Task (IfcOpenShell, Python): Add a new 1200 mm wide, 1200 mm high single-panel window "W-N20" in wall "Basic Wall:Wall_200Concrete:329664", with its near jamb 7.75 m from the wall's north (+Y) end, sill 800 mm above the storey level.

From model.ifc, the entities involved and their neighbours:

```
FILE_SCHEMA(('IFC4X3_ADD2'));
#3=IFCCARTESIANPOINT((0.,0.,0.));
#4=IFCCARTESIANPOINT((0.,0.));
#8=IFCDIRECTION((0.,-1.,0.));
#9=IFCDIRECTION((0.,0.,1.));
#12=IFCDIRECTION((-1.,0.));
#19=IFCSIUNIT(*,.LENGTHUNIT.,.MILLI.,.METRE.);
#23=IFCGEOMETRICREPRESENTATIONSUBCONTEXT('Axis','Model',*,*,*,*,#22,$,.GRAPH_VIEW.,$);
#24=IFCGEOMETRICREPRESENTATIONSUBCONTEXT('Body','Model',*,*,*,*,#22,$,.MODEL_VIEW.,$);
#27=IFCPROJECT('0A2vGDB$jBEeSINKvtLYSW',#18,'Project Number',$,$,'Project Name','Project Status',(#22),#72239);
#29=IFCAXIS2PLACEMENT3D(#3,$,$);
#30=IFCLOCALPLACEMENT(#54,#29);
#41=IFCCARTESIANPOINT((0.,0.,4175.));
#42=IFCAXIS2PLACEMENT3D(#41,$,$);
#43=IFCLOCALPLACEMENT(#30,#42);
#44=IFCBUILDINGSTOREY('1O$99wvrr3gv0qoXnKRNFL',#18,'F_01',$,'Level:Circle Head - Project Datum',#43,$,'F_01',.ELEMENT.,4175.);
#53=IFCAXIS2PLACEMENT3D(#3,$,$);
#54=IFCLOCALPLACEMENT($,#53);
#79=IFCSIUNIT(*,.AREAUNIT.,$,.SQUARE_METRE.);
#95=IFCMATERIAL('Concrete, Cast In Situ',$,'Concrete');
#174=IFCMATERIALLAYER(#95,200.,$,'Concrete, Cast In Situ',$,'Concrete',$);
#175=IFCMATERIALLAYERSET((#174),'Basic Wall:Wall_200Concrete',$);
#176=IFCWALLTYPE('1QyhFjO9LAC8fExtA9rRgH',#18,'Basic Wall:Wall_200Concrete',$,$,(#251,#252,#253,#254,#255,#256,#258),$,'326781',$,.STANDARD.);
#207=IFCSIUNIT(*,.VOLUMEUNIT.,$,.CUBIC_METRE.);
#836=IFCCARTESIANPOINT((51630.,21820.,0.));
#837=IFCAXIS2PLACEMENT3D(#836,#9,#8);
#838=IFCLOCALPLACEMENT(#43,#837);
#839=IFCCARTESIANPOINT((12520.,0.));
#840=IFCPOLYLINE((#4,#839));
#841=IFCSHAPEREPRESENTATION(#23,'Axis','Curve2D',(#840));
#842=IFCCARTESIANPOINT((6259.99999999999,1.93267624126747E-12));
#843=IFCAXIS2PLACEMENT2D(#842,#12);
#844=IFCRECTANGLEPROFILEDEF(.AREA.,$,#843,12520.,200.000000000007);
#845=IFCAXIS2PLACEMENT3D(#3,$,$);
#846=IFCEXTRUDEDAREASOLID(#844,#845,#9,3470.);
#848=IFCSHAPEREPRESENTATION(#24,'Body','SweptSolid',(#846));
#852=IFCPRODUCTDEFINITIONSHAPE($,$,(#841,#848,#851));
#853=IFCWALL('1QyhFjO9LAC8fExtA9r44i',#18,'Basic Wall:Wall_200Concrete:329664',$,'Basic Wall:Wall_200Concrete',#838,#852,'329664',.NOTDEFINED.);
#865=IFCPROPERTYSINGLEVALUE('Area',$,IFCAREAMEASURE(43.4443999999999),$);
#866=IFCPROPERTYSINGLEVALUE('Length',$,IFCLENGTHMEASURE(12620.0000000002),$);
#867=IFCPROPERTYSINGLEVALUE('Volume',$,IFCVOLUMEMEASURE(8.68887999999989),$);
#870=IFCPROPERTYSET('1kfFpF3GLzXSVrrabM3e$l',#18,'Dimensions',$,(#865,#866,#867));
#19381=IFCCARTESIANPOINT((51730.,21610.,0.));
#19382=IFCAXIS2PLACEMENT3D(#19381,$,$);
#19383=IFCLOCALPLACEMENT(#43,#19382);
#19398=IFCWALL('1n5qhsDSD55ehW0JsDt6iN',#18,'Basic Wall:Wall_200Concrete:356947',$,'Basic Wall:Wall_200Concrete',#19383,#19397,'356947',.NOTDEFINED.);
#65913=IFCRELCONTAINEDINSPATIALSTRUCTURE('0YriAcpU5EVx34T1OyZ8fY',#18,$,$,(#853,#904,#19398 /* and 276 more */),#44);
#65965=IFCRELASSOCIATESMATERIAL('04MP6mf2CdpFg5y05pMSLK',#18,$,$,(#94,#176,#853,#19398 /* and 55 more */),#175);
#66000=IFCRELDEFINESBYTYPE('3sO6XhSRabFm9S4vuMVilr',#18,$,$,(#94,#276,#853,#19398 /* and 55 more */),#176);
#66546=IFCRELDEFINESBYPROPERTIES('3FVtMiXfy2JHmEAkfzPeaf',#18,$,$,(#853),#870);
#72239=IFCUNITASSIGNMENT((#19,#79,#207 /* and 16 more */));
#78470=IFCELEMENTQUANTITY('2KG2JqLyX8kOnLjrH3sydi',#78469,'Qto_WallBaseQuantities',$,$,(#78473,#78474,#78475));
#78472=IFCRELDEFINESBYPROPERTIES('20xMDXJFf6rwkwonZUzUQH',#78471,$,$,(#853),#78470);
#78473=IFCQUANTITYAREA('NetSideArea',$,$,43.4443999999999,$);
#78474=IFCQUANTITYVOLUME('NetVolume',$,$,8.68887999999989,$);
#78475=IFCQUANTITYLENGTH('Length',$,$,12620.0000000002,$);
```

```python
import numpy as np
import ifcopenshell
import ifcopenshell.api.feature
import ifcopenshell.api.geometry
import ifcopenshell.api.pset
import ifcopenshell.api.root
import ifcopenshell.api.spatial
import ifcopenshell.geom
import ifcopenshell.util.element
import ifcopenshell.util.placement
import ifcopenshell.util.representation
import ifcopenshell.util.shape
import ifcopenshell.util.unit

model = ifcopenshell.open("model.ifc")
unit_scale = ifcopenshell.util.unit.calculate_unit_scale(model)
area_scale = ifcopenshell.util.unit.calculate_unit_scale(model, "AREAUNIT")
volume_scale = ifcopenshell.util.unit.calculate_unit_scale(model, "VOLUMEUNIT")
settings = ifcopenshell.geom.settings()


def volume(element):
    """Net volume in cubic metres, openings subtracted."""
    shape = ifcopenshell.geom.create_shape(settings, element)
    return ifcopenshell.util.shape.get_volume(shape.geometry)


wall = model.by_guid("1QyhFjO9LAC8fExtA9r44i")
storey = ifcopenshell.util.element.get_container(wall, ifc_class="IfcBuildingStorey")
context = ifcopenshell.util.representation.get_context(model, "Model", "Body", "MODEL_VIEW")
before = volume(wall)

width, height, from_end, sill = 1.2, 1.2, 7.75, 0.8  # metres

# The wall runs along its own X axis, and the end named is its -X end.
wall_shape = ifcopenshell.geom.create_shape(settings, wall)
x, y, z = ifcopenshell.util.shape.get_vertices(wall_shape.geometry).T
start = x.min() + from_end
face, thickness = float(y.min()), float(y.max() - y.min())
wall_matrix = ifcopenshell.util.placement.get_local_placement(wall.ObjectPlacement)
level = ifcopenshell.util.placement.get_local_placement(storey.ObjectPlacement)[2, 3]


def in_wall(x, y):
    """Placement at x, y metres in the wall's axes, at sill height."""
    matrix = wall_matrix.copy()
    matrix[:, 3] = wall_matrix @ np.array([x / unit_scale, y / unit_scale, 0.0, 1.0])
    matrix[2, 3] = level + sill / unit_scale
    return matrix


# Opening: a box that overshoots both wall faces by 50 mm.
opening = ifcopenshell.api.root.create_entity(model, ifc_class="IfcOpeningElement", predefined_type="OPENING")
box = ifcopenshell.api.geometry.add_wall_representation(
    model, context=context, length=width, height=height, thickness=thickness + 0.1
)
ifcopenshell.api.geometry.assign_representation(model, product=opening, representation=box)
ifcopenshell.api.geometry.edit_object_placement(model, product=opening, matrix=in_wall(start, face - 0.05), is_si=False)
ifcopenshell.api.feature.add_feature(model, feature=opening, element=wall)

window = ifcopenshell.api.root.create_entity(model, ifc_class="IfcWindow", name="W-N20", predefined_type="WINDOW")
window.OverallWidth, window.OverallHeight = width / unit_scale, height / unit_scale
window.PartitioningType = "SINGLE_PANEL"
body = ifcopenshell.api.geometry.add_window_representation(
    model,
    context=context,
    overall_width=window.OverallWidth,
    overall_height=window.OverallHeight,
    partition_type="SINGLE_PANEL",
)
ifcopenshell.api.geometry.assign_representation(model, product=window, representation=body)
ifcopenshell.api.spatial.assign_container(model, products=[window], relating_structure=storey)
ifcopenshell.api.feature.add_filling(model, opening=opening, element=window)

# Centre the window in the wall's thickness.
ifcopenshell.api.geometry.edit_object_placement(model, product=window, matrix=in_wall(start, face), is_si=False)
window_shape = ifcopenshell.geom.create_shape(settings, window)
depth = ifcopenshell.util.shape.get_vertices(window_shape.geometry)[:, 1]
offset = face + thickness / 2 - (depth.min() + depth.max()) / 2
ifcopenshell.api.geometry.edit_object_placement(model, product=window, matrix=in_wall(start, offset), is_si=False)

after = volume(wall)

# Update the wall's stored quantities.
pset = model.by_id(ifcopenshell.util.element.get_pset(wall, "Dimensions", should_inherit=False)["id"])
ifcopenshell.api.pset.edit_pset(model, pset=pset, properties={
    "Area": model.create_entity("IfcAreaMeasure", after / thickness / area_scale),
    "Volume": model.create_entity("IfcVolumeMeasure", after / volume_scale),
})
qto = model.by_id(ifcopenshell.util.element.get_pset(wall, "Qto_WallBaseQuantities", should_inherit=False)["id"])
ifcopenshell.api.pset.edit_qto(model, qto=qto, properties={
    "NetSideArea": after / thickness / area_scale,
    "NetVolume": after / volume_scale,
})

print(f"wall volume {before:.3f} -> {after:.3f} m3")

model.write("model_v2.ifc")
```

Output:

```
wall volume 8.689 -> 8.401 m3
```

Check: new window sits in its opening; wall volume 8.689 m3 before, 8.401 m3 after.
